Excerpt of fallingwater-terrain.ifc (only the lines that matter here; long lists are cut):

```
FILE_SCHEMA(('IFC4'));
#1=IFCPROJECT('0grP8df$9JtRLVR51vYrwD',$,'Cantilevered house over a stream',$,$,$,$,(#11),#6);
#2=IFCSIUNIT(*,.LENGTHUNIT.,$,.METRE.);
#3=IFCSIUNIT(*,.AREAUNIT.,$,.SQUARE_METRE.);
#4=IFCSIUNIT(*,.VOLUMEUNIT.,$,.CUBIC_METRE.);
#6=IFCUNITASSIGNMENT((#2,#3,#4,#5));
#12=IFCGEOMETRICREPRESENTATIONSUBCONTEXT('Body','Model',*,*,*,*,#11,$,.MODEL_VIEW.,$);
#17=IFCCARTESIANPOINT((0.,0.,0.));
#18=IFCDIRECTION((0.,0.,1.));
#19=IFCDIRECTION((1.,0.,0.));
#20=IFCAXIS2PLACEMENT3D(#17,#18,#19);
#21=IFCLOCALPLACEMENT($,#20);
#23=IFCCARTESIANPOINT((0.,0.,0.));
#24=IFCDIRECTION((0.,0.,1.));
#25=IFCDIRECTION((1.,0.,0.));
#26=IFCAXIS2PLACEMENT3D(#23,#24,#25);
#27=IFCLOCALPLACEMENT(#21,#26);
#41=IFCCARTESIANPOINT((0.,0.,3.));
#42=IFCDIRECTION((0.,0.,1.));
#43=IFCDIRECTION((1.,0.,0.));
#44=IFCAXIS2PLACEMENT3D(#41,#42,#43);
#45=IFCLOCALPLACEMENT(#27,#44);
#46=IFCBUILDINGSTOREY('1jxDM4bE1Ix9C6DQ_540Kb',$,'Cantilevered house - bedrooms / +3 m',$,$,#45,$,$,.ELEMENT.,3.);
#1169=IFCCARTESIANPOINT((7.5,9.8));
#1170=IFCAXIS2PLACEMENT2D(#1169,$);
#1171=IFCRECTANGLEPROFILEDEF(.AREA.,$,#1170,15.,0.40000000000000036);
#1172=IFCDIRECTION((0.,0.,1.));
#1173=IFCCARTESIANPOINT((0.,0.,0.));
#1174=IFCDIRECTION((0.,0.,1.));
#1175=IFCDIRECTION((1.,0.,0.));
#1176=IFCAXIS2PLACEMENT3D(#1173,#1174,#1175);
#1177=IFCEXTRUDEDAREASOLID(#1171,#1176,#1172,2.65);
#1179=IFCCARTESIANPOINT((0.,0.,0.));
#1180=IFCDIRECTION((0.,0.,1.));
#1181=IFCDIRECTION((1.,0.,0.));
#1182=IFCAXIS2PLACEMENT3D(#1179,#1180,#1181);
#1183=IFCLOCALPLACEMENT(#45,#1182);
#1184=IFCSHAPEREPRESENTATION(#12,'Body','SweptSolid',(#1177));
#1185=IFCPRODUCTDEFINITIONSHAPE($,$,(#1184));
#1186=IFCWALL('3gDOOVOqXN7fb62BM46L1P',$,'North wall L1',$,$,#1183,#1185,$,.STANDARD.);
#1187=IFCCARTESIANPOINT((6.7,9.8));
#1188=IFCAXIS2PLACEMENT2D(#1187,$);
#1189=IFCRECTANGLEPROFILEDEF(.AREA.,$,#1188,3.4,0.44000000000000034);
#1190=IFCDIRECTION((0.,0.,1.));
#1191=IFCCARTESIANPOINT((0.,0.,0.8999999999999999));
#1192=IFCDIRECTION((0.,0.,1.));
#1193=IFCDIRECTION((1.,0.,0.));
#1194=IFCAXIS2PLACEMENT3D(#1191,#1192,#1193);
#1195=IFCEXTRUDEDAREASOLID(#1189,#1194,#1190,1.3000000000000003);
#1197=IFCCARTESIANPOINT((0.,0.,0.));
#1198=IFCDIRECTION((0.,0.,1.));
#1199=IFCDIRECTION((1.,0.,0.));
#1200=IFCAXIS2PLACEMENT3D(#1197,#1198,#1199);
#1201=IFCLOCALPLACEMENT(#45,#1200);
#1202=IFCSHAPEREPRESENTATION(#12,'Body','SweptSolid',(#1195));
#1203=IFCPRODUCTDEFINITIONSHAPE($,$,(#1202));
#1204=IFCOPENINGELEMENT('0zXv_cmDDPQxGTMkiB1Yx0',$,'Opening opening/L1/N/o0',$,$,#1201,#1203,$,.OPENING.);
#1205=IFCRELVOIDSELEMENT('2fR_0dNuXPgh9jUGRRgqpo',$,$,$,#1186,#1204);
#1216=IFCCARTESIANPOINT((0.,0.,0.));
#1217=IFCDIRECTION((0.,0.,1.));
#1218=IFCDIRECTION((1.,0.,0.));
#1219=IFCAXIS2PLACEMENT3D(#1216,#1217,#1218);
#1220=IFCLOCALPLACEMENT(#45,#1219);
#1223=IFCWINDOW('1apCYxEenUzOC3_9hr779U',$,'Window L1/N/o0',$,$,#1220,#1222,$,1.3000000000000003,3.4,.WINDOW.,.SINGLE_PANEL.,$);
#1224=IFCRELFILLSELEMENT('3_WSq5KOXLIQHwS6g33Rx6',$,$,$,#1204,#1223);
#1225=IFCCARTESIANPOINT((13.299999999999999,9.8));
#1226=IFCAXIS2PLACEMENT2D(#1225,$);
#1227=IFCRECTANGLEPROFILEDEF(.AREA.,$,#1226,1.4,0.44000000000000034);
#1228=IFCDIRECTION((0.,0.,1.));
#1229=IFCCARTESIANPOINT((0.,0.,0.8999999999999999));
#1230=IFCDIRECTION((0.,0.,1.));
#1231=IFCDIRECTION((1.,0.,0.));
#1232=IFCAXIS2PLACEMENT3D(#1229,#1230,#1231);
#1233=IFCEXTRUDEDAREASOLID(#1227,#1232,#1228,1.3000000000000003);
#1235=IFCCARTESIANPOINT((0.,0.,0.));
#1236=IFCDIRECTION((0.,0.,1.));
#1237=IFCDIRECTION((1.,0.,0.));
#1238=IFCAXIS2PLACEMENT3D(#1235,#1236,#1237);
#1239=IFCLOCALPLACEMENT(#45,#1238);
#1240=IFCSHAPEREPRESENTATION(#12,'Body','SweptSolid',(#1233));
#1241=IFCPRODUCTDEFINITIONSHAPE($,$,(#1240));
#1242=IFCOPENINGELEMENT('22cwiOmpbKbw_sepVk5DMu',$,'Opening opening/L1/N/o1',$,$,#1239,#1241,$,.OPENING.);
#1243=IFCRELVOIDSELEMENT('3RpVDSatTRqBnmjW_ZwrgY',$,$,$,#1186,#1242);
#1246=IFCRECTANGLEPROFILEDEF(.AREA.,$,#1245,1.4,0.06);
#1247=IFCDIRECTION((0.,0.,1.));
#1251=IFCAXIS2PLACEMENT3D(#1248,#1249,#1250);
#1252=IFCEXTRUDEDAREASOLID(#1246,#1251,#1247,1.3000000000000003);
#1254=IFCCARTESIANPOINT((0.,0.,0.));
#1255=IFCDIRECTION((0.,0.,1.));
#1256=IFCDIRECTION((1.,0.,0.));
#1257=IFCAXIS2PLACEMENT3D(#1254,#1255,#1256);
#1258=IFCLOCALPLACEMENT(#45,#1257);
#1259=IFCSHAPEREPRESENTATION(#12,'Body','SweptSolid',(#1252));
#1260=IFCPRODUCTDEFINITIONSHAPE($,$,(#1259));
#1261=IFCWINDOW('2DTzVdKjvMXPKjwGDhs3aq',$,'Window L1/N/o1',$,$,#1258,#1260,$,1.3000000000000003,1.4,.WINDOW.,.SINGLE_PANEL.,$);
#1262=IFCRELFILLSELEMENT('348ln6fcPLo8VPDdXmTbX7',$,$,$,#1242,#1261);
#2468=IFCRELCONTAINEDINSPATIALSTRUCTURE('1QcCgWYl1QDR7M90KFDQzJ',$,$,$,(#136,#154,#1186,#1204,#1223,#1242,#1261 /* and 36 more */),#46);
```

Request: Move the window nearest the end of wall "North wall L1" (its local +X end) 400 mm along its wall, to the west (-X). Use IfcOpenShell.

```python
import ifcopenshell
import ifcopenshell.api.geometry
import ifcopenshell.util.placement
import ifcopenshell.util.unit

model = ifcopenshell.open("fallingwater-terrain.ifc")
unit_scale = ifcopenshell.util.unit.calculate_unit_scale(model)

window = model.by_guid("2DTzVdKjvMXPKjwGDhs3aq")
opening = window.FillsVoids[0].RelatingOpeningElement
wall = opening.VoidsElements[0].RelatingBuildingElement

wall_matrix = ifcopenshell.util.placement.get_local_placement(wall.ObjectPlacement)
shift = wall_matrix[:3, 0] * -0.4 / unit_scale
before = ifcopenshell.util.placement.get_local_placement(window.ObjectPlacement)[:3, 3].copy()

# The window is not placed relative to its opening, so move both.
for product in (opening, window):
    matrix = ifcopenshell.util.placement.get_local_placement(product.ObjectPlacement)
    matrix[:3, 3] += shift
    ifcopenshell.api.geometry.edit_object_placement(model, product=product, matrix=matrix, is_si=False)

after = ifcopenshell.util.placement.get_local_placement(window.ObjectPlacement)[:3, 3]
print("window moved by", (after - before).round(3) + 0.0)

model.write("fallingwater-terrain_updated.ifc")
```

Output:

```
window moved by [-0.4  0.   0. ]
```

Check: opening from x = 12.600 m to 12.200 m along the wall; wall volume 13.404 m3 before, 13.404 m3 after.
